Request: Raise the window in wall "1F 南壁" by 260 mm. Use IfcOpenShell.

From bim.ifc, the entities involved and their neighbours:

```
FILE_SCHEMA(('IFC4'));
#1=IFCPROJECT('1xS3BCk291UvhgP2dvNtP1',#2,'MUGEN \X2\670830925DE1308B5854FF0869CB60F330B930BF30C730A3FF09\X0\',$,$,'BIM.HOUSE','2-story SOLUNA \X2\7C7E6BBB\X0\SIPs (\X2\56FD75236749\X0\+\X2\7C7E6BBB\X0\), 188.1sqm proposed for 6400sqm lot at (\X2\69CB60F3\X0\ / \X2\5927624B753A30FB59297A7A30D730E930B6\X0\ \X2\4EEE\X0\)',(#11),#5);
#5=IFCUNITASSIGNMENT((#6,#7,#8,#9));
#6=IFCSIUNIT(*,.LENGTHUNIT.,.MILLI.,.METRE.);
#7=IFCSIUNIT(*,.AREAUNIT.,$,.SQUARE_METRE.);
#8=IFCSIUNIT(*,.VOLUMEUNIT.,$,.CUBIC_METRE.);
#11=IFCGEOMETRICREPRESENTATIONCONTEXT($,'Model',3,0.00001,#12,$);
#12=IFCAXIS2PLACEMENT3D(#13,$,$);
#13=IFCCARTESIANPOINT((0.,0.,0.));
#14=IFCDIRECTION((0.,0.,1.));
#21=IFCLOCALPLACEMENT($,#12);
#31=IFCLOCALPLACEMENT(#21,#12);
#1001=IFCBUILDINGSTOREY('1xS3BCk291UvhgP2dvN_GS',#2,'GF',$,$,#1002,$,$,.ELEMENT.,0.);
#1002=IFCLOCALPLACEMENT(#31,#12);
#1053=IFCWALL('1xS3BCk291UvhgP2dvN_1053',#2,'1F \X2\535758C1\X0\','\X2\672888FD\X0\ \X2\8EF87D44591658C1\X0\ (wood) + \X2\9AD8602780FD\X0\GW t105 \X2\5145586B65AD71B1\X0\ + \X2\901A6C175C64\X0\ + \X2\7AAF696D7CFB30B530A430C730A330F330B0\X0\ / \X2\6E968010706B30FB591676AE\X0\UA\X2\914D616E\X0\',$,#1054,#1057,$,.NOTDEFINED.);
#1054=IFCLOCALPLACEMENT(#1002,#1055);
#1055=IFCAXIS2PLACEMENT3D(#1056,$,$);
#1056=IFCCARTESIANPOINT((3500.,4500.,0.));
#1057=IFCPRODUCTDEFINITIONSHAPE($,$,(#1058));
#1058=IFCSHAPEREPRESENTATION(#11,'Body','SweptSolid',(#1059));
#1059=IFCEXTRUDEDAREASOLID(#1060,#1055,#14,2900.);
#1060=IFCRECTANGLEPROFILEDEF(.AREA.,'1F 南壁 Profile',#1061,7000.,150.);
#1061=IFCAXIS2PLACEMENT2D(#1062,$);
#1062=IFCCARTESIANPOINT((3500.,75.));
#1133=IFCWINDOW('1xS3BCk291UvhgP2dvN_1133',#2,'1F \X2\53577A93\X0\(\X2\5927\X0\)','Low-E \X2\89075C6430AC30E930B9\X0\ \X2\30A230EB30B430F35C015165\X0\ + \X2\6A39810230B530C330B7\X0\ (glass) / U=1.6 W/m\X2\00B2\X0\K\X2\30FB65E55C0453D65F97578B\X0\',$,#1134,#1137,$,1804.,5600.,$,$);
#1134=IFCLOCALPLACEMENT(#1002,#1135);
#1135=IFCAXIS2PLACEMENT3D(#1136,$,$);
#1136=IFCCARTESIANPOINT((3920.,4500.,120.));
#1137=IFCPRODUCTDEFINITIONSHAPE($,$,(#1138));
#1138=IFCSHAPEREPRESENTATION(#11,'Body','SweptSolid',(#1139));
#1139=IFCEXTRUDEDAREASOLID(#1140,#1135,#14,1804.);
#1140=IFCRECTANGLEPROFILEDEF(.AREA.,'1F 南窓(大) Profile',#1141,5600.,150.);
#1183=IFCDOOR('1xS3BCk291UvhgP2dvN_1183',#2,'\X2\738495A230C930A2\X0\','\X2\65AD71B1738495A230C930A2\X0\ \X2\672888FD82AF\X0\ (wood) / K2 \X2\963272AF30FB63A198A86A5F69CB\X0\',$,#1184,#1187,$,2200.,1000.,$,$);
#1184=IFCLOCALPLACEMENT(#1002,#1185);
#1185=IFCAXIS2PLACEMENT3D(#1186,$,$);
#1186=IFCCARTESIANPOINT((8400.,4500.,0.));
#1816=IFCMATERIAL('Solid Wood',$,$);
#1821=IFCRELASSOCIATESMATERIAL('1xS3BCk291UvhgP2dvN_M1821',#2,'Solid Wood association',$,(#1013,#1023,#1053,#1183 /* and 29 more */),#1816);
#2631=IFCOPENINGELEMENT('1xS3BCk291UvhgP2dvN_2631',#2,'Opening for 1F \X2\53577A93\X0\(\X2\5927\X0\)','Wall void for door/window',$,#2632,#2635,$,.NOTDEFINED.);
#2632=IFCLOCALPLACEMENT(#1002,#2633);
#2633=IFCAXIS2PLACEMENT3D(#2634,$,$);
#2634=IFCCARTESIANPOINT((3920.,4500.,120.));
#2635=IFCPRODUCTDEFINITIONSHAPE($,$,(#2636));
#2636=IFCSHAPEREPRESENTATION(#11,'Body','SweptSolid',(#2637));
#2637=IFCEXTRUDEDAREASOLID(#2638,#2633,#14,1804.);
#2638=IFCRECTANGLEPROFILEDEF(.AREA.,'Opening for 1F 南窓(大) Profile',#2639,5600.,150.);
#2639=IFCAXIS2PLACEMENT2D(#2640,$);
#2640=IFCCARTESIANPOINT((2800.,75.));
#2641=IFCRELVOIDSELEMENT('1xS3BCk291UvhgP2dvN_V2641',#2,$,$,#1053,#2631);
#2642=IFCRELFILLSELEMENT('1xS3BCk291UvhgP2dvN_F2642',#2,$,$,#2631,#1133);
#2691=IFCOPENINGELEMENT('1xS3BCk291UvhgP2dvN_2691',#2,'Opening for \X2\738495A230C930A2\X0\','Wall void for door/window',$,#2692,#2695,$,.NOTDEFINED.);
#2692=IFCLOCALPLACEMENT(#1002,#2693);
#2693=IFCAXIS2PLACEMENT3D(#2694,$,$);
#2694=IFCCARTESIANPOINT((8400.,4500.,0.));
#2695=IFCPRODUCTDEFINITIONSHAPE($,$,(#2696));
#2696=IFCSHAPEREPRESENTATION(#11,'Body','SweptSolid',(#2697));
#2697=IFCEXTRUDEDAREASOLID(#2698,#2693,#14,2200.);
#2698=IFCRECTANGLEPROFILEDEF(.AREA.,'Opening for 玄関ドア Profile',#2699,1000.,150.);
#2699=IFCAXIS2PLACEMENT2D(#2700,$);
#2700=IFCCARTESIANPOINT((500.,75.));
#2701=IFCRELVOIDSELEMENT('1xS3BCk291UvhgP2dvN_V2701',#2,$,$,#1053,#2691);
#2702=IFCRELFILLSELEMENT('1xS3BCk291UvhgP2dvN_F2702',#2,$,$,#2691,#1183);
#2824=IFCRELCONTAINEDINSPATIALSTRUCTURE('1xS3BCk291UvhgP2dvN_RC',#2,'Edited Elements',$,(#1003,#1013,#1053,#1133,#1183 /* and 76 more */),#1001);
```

```python
import numpy as np
import ifcopenshell
import ifcopenshell.api.geometry
import ifcopenshell.util.placement
import ifcopenshell.util.unit

model = ifcopenshell.open("bim.ifc")
unit_scale = ifcopenshell.util.unit.calculate_unit_scale(model)

window = model.by_guid("1xS3BCk291UvhgP2dvN_1133")
opening = window.FillsVoids[0].RelatingOpeningElement
dz = 0.26 / unit_scale

shift = np.array([0.0, 0.0, dz])
# The window is not placed relative to its opening, so move both.
for product in (opening, window):
    matrix = ifcopenshell.util.placement.get_local_placement(product.ObjectPlacement)
    matrix[:3, 3] += shift
    ifcopenshell.api.geometry.edit_object_placement(model, product=product, matrix=matrix, is_si=False)

print(f"moved by {dz * unit_scale:+.3f} m")

model.write("bim_edited.ifc")
```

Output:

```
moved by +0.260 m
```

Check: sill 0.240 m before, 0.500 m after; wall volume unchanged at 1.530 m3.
